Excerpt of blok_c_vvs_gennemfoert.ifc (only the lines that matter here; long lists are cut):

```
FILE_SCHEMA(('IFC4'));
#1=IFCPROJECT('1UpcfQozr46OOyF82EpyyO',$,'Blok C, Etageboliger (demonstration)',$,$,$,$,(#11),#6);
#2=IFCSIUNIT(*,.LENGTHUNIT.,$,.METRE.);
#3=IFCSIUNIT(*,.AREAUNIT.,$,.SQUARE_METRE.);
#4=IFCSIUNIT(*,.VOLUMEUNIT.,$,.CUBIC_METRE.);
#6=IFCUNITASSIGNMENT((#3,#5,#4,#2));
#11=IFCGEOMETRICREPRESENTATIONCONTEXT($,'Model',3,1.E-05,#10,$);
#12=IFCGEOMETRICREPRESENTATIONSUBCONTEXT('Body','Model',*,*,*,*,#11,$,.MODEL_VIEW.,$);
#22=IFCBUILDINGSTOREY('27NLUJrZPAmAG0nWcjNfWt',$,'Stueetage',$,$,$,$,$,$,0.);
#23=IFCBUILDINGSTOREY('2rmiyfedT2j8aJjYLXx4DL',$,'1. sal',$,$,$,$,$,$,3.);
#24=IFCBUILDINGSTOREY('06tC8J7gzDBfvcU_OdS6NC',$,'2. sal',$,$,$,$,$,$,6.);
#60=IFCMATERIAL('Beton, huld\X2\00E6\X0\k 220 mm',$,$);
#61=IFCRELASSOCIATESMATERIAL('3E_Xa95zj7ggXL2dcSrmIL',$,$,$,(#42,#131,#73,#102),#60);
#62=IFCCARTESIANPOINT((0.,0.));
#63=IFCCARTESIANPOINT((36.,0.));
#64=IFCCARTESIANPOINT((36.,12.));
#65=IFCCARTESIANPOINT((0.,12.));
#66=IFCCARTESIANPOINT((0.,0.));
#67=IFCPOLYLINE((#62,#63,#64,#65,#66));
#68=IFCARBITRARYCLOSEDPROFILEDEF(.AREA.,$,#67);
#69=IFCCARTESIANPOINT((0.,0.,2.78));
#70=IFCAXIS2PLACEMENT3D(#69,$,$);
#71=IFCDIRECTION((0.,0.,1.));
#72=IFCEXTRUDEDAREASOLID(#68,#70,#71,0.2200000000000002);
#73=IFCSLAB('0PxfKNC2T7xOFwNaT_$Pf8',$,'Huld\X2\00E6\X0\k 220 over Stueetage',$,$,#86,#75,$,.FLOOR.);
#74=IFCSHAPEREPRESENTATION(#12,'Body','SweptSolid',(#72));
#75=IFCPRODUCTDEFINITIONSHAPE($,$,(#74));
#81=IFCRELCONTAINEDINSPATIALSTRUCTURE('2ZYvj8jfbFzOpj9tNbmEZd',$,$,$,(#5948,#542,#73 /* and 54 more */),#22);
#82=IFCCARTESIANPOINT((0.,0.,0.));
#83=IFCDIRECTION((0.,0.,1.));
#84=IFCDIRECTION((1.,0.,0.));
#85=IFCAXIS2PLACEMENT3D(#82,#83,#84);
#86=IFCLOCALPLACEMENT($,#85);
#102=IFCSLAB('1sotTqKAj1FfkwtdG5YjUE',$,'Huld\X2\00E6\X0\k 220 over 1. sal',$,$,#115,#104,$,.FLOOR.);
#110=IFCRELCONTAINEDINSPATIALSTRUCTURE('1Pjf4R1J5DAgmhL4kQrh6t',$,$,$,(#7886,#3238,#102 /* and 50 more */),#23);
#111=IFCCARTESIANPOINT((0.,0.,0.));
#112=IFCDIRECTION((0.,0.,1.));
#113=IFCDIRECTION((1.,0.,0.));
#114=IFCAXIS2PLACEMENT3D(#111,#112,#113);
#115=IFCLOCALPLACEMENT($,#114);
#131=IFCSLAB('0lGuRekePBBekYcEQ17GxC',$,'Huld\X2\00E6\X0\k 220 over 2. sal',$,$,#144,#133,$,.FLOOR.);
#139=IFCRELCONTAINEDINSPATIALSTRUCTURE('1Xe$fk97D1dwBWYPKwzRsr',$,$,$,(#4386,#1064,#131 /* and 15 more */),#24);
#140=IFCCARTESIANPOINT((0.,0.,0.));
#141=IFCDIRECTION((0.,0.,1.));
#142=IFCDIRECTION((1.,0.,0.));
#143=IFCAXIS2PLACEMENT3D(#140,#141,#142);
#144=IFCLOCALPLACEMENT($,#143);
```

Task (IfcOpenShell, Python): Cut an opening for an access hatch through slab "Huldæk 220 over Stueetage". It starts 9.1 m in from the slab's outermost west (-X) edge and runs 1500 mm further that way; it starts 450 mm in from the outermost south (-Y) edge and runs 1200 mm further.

```python
import numpy as np
import ifcopenshell
import ifcopenshell.api.feature
import ifcopenshell.api.geometry
import ifcopenshell.api.root
import ifcopenshell.geom
import ifcopenshell.util.placement
import ifcopenshell.util.representation
import ifcopenshell.util.shape
import ifcopenshell.util.unit

model = ifcopenshell.open("blok_c_vvs_gennemfoert.ifc")
unit_scale = ifcopenshell.util.unit.calculate_unit_scale(model)
settings = ifcopenshell.geom.settings()


def volume(element):
    """Net volume in cubic metres, openings subtracted."""
    shape = ifcopenshell.geom.create_shape(settings, element)
    return ifcopenshell.util.shape.get_volume(shape.geometry)


slab = model.by_id(73)
before = volume(slab)

# Extent in the slab's own axes, in metres. The edges named are its -X and -Y sides.
slab_shape = ifcopenshell.geom.create_shape(settings, slab)
vertices = ifcopenshell.util.shape.get_vertices(slab_shape.geometry)
x_min, y_min, bottom = vertices.min(axis=0)
top = vertices[:, 2].max()

opening = ifcopenshell.api.root.create_entity(model, ifc_class="IfcOpeningElement", name="Access hatch opening", predefined_type="OPENING")
context = ifcopenshell.util.representation.get_context(model, "Model", "Body", "MODEL_VIEW")
width, depth = 1.5, 1.2
outline = [(0.0, 0.0), (width, 0.0), (width, depth), (0.0, depth), (0.0, 0.0)]
# Overshoot both faces by 50 mm so the cut is clean.
shape = ifcopenshell.api.geometry.add_slab_representation(
    model, context=context, depth=top - bottom + 0.1, polyline=outline
)
ifcopenshell.api.geometry.assign_representation(model, product=opening, representation=shape)

matrix = ifcopenshell.util.placement.get_local_placement(slab.ObjectPlacement)
matrix[:, 3] = matrix @ np.append(np.array([x_min + 9.1, y_min + 0.45, bottom - 0.05]) / unit_scale, 1.0)
ifcopenshell.api.geometry.edit_object_placement(model, product=opening, matrix=matrix, is_si=False)
ifcopenshell.api.feature.add_feature(model, feature=opening, element=slab)

after = volume(slab)

print(f"slab volume {before:.3f} -> {after:.3f} m3")

model.write("blok_c_vvs_gennemfoert_edited.ifc")
```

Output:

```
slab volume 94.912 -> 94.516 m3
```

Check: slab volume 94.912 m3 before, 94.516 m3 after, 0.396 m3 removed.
